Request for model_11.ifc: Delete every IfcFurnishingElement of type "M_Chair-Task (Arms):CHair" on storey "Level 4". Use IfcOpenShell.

First a look at what the model holds.

```python
import ifcopenshell
import ifcopenshell.util.element

model = ifcopenshell.open("model_11.ifc")
print(model.schema)
storey = next(s for s in model.by_type("IfcBuildingStorey") if s.Name == "Level 4")
furniture = [e for e in ifcopenshell.util.element.get_decomposition(storey) if e.is_a("IfcFurnishingElement")]
seen = {}
for e in furniture:
    element_type = ifcopenshell.util.element.get_type(e)
    name = element_type.Name if element_type not in (None, e) else None
    seen[name] = seen.get(name, 0) + 1
for name, count in sorted(seen.items(), key=str):
    print(count, "x", name)
```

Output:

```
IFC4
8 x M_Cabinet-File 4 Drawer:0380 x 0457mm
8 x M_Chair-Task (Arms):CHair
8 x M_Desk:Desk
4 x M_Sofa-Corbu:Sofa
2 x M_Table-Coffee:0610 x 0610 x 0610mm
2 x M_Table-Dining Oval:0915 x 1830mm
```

```python
import ifcopenshell
import ifcopenshell.api.root
import ifcopenshell.util.element

model = ifcopenshell.open("model_11.ifc")

storey = next(s for s in model.by_type("IfcBuildingStorey") if s.Name == "Level 4")
furniture = [e for e in ifcopenshell.util.element.get_decomposition(storey) if e.is_a("IfcFurnishingElement")]
targets = [e for e in furniture if (t := ifcopenshell.util.element.get_type(e)) not in (None, e) and t.Name == "M_Chair-Task (Arms):CHair"]

for e in targets:
    ifcopenshell.api.root.remove_product(model, product=e)
print(len(targets), "removed")

model.write("model_11_updated.ifc")
```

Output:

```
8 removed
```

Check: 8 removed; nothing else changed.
